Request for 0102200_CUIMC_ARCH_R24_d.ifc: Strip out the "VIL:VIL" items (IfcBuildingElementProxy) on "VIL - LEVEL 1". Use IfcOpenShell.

First a look at what the model holds.

```python
import ifcopenshell
import ifcopenshell.util.element

model = ifcopenshell.open("0102200_CUIMC_ARCH_R24_d.ifc")
print(model.schema)
storey = next(s for s in model.by_type("IfcBuildingStorey") if s.Name == "VIL - LEVEL 1")
proxies = [e for e in ifcopenshell.util.element.get_decomposition(storey) if e.is_a("IfcBuildingElementProxy")]
seen = {}
for e in proxies:
    element_type = ifcopenshell.util.element.get_type(e)
    name = element_type.Name if element_type not in (None, e) else None
    seen[name] = seen.get(name, 0) + 1
for name, count in sorted(seen.items(), key=str):
    print(count, "x", name)
```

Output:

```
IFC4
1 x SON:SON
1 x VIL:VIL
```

```python
import ifcopenshell
import ifcopenshell.api.root
import ifcopenshell.util.element

model = ifcopenshell.open("0102200_CUIMC_ARCH_R24_d.ifc")

storey = next(s for s in model.by_type("IfcBuildingStorey") if s.Name == "VIL - LEVEL 1")
proxies = [e for e in ifcopenshell.util.element.get_decomposition(storey) if e.is_a("IfcBuildingElementProxy")]
targets = [e for e in proxies if (t := ifcopenshell.util.element.get_type(e)) not in (None, e) and t.Name == "VIL:VIL"]

for e in targets:
    ifcopenshell.api.root.remove_product(model, product=e)
print(len(targets), "removed")

model.write("0102200_CUIMC_ARCH_R24_d_v2.ifc")
```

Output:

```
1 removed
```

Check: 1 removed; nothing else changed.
